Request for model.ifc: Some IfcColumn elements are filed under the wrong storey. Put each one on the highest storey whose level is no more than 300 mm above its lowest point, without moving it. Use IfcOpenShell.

First a look at what the model holds.

```python
import ifcopenshell
import ifcopenshell.util.element
import ifcopenshell.util.placement

model = ifcopenshell.open("model.ifc")
print(model.schema)
for storey in model.by_type("IfcBuildingStorey"):
    level = ifcopenshell.util.placement.get_storey_elevation(storey)
    count = sum(e.is_a("IfcColumn") for e in ifcopenshell.util.element.get_contained(storey))
    print(storey.id(), storey.Name, round(level, 3), count, sep=" | ")
```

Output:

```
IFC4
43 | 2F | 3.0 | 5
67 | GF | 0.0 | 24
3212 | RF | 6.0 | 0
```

```python
import ifcopenshell
import ifcopenshell.api.spatial
import ifcopenshell.geom
import ifcopenshell.util.element
import ifcopenshell.util.placement
import ifcopenshell.util.shape
import ifcopenshell.util.unit

model = ifcopenshell.open("model.ifc")
unit_scale = ifcopenshell.util.unit.calculate_unit_scale(model)
settings = ifcopenshell.geom.settings()

levels = sorted(
    ((ifcopenshell.util.placement.get_storey_elevation(s) * unit_scale, s) for s in model.by_type("IfcBuildingStorey")),
    key=lambda pair: pair[0],
)

for e in model.by_type("IfcColumn"):
    current = e.ContainedInStructure[0].RelatingStructure if e.ContainedInStructure else None
    if current is None or not current.is_a("IfcBuildingStorey"):
        continue
    shape = ifcopenshell.geom.create_shape(settings, e)
    bottom = ifcopenshell.util.shape.get_shape_bottom_elevation(shape, shape.geometry)
    below = [s for level, s in levels if level <= bottom + 0.3]
    storey = below[-1] if below else levels[0][1]
    if storey != current:
        # assign_container keeps the world position.
        ifcopenshell.api.spatial.assign_container(model, products=[e], relating_structure=storey)
        print(e.id(), current.Name, "->", storey.Name)

model.write("model_edited.ifc")
```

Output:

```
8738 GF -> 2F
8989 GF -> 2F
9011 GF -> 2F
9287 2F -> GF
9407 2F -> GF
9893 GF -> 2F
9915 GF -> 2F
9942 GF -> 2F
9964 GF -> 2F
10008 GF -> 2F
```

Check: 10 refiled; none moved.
